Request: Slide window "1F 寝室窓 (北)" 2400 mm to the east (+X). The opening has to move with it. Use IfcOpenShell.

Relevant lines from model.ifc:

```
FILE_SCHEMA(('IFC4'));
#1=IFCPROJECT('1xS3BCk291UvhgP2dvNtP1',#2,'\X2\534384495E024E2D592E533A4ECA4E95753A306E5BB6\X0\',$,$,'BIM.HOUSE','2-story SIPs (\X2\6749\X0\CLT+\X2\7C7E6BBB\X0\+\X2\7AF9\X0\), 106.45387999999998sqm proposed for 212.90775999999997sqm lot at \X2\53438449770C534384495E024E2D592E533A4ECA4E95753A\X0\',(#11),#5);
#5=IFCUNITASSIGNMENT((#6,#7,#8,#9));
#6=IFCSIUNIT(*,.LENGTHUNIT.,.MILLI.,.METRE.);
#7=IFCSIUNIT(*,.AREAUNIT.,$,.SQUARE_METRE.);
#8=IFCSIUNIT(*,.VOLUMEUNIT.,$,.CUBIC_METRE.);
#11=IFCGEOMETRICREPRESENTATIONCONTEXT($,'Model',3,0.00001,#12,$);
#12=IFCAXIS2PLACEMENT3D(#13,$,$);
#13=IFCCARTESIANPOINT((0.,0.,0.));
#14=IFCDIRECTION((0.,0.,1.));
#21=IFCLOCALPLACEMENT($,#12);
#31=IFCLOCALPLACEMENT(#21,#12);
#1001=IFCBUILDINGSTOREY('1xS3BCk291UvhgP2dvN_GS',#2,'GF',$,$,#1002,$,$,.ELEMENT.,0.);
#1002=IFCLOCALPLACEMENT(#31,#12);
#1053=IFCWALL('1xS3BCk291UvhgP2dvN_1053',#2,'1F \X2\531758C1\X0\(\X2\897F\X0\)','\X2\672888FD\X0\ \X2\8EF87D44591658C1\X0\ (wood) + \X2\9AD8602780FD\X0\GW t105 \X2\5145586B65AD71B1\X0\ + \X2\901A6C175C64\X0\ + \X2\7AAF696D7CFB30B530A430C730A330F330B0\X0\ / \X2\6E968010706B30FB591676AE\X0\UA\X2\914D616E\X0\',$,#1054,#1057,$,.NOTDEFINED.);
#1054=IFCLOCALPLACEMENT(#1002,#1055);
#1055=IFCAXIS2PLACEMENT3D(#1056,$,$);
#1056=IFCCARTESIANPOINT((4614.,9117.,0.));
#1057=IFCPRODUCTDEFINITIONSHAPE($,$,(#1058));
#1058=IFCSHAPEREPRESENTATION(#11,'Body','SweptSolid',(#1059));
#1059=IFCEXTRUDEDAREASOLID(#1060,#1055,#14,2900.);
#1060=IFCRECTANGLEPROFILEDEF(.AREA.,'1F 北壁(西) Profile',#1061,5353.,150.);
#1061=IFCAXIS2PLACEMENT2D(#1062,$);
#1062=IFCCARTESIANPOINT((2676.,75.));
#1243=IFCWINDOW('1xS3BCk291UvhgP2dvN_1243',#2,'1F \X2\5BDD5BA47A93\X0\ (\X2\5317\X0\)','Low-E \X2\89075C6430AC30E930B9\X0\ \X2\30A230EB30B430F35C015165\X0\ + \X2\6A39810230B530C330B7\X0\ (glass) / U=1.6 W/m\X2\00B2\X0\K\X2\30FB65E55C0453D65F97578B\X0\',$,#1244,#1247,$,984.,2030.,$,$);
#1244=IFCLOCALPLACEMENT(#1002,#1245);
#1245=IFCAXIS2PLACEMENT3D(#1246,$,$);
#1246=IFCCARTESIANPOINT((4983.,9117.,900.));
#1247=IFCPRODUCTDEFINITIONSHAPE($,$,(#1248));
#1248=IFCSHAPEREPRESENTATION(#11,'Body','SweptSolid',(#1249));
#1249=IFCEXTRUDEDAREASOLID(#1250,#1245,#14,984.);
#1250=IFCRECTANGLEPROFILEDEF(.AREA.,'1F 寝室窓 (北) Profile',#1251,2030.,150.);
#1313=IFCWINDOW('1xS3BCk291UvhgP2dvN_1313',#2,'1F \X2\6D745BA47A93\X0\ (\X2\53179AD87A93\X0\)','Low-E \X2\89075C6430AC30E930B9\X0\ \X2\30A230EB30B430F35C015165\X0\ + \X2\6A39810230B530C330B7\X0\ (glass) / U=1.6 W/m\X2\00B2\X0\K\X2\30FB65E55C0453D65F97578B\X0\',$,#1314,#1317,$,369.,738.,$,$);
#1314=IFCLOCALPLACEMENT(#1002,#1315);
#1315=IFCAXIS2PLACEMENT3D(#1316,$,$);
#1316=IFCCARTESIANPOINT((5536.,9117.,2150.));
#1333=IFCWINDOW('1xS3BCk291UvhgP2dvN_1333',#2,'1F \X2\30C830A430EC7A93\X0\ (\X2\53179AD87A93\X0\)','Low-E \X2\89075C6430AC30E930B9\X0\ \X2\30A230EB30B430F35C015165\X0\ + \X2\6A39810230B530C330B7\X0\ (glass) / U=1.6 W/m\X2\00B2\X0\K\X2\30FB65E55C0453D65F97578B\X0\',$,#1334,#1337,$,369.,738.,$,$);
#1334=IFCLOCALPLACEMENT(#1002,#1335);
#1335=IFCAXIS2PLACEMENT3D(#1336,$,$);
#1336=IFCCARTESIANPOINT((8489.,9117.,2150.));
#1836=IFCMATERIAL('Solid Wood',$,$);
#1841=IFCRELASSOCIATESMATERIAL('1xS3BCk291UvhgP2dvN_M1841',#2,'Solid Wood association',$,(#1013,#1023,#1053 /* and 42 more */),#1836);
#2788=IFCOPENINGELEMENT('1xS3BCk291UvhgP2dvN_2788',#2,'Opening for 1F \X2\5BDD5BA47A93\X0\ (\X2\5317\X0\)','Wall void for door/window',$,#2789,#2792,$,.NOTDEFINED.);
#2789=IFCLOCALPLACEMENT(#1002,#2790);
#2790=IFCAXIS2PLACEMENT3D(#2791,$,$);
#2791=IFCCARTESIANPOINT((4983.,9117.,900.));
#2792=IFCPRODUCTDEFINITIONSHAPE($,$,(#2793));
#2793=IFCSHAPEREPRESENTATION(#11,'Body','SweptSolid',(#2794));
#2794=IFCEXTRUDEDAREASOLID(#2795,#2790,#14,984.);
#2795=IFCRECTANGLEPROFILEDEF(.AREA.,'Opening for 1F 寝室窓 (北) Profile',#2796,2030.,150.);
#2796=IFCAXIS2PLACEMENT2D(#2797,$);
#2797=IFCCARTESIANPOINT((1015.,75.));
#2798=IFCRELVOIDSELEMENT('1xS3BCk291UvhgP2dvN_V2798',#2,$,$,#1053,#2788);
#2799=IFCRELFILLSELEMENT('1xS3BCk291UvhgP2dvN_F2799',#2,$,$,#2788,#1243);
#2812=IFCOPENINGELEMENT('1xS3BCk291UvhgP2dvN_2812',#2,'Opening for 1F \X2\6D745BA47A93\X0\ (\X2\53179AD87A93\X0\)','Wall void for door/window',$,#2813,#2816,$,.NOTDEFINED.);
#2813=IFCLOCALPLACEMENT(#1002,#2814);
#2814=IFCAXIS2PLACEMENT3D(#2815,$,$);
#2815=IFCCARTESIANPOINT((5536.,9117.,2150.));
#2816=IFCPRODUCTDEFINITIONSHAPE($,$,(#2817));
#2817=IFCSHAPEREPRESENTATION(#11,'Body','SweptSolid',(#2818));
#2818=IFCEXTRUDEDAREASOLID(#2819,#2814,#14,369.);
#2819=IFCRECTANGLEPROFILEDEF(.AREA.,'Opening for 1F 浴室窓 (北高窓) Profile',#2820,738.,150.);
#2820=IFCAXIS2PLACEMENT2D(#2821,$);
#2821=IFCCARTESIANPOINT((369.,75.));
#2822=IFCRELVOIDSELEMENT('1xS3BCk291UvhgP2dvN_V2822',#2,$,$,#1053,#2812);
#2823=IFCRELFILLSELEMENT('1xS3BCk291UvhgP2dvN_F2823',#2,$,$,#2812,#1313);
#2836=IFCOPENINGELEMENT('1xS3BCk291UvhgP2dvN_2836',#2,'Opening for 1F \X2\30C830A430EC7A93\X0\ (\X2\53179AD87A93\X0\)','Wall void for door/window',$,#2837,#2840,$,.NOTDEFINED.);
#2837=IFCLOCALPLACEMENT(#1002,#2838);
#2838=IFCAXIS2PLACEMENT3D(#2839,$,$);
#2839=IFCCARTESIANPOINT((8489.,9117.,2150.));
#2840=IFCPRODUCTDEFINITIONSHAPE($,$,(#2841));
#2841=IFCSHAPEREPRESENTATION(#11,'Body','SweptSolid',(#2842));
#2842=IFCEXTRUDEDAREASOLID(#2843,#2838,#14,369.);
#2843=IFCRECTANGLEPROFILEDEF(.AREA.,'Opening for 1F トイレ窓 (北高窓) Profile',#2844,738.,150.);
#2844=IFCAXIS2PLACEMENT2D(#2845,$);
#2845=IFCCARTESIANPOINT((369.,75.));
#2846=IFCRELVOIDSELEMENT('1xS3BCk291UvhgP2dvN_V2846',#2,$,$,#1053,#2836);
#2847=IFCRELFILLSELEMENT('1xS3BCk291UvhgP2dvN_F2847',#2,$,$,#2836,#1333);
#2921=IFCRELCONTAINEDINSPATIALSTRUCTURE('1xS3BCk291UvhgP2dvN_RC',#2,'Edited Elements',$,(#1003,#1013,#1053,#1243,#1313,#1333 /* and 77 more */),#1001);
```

```python
import ifcopenshell
import ifcopenshell.api.geometry
import ifcopenshell.util.placement
import ifcopenshell.util.unit

model = ifcopenshell.open("model.ifc")
unit_scale = ifcopenshell.util.unit.calculate_unit_scale(model)

window = model.by_id(1243)
opening = window.FillsVoids[0].RelatingOpeningElement
wall = opening.VoidsElements[0].RelatingBuildingElement

wall_matrix = ifcopenshell.util.placement.get_local_placement(wall.ObjectPlacement)
shift = wall_matrix[:3, 0] * 2.4 / unit_scale
before = ifcopenshell.util.placement.get_local_placement(window.ObjectPlacement)[:3, 3].copy()

# The window is not placed relative to its opening, so move both.
for product in (opening, window):
    matrix = ifcopenshell.util.placement.get_local_placement(product.ObjectPlacement)
    matrix[:3, 3] += shift
    ifcopenshell.api.geometry.edit_object_placement(model, product=product, matrix=matrix, is_si=False)

after = ifcopenshell.util.placement.get_local_placement(window.ObjectPlacement)[:3, 3]
print("window moved by", (after - before).round(3) + 0.0)

model.write("model_rev.ifc")
```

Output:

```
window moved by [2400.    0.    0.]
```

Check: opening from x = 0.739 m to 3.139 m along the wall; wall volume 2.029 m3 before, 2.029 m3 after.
